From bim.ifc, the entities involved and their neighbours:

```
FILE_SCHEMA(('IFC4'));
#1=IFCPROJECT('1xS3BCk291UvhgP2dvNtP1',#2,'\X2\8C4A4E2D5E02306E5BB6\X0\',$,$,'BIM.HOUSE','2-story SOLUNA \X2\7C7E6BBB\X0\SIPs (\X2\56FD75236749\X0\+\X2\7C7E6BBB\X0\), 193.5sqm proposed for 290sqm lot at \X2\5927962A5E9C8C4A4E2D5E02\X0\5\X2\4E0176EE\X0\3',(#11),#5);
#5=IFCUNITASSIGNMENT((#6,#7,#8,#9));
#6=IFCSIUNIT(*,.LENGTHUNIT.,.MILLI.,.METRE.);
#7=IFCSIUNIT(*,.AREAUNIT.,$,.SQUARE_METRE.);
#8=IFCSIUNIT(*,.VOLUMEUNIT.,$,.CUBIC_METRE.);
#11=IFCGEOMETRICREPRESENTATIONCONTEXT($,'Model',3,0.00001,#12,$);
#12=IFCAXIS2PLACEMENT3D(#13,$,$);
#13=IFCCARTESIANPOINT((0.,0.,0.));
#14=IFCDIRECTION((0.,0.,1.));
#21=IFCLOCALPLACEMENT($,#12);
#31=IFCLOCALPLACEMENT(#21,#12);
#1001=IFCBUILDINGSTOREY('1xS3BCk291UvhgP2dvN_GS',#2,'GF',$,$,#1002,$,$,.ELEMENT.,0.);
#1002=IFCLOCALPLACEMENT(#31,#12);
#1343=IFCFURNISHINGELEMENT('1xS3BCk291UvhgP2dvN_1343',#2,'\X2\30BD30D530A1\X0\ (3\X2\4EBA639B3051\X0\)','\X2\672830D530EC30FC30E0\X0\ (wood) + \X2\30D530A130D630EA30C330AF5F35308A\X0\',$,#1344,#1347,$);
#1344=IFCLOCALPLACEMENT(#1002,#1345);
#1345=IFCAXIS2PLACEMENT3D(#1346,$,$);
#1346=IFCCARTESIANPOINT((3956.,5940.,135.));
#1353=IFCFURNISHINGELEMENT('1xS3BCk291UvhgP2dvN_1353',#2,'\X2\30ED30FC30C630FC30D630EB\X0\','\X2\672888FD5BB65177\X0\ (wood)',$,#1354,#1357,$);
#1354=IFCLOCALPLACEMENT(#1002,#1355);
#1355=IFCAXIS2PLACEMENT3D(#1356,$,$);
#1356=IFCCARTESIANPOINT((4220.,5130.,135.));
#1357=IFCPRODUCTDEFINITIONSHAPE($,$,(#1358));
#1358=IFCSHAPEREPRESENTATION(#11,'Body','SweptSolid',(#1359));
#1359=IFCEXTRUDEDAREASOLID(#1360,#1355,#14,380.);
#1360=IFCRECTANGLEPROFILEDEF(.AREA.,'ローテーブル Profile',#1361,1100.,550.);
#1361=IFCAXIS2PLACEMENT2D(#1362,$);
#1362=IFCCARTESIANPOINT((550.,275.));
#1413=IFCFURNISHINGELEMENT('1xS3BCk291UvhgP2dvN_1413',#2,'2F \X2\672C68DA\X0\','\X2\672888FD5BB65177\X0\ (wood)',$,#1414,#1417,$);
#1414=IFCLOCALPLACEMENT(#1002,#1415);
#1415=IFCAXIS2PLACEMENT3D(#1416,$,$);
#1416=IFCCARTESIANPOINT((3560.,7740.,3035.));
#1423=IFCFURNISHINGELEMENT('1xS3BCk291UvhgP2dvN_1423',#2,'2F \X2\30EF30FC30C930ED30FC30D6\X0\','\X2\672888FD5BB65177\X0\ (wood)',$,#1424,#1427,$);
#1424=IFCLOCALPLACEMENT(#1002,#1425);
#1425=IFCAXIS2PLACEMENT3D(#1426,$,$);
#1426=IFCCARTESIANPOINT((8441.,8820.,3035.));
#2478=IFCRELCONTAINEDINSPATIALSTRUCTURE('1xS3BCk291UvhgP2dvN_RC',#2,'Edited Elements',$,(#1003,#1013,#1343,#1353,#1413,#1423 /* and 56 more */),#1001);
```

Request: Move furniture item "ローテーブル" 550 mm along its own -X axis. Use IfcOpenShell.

```python
import ifcopenshell
import ifcopenshell.api.geometry
import ifcopenshell.util.placement
import ifcopenshell.util.unit

model = ifcopenshell.open("bim.ifc")
unit_scale = ifcopenshell.util.unit.calculate_unit_scale(model)

item = model.by_id(1353)
matrix = ifcopenshell.util.placement.get_local_placement(item.ObjectPlacement)
matrix[:3, 3] -= matrix[:3, 0] * 0.55 / unit_scale
ifcopenshell.api.geometry.edit_object_placement(model, product=item, matrix=matrix, is_si=False)

print(ifcopenshell.util.placement.get_local_placement(item.ObjectPlacement).round(3) + 0.0)

model.write("bim_v2.ifc")
```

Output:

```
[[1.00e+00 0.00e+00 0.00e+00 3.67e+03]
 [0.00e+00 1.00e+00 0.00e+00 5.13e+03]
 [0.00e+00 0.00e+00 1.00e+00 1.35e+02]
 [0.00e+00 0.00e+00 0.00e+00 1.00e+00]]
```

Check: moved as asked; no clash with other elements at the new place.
